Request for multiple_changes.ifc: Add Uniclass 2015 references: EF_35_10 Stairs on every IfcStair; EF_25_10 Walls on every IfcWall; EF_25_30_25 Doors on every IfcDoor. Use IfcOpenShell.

First a look at what the model holds.

```python
import ifcopenshell

model = ifcopenshell.open("multiple_changes.ifc")
print(model.schema)
print("classifications:", [c.Name for c in model.by_type("IfcClassification")])
for ifc_class in ("IfcDoor", "IfcRoof", "IfcStair", "IfcWall", "IfcWindow"):
    print(ifc_class, len(model.by_type(ifc_class)))
```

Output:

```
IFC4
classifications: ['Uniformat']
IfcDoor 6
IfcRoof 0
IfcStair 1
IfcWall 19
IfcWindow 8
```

```python
import ifcopenshell
import ifcopenshell.api.classification

model = ifcopenshell.open("multiple_changes.ifc")

system = ifcopenshell.api.classification.add_classification(model, classification="Uniclass 2015")

codes = {
    "IfcStair": ("EF_35_10", "Stairs"),
    "IfcWall": ("EF_25_10", "Walls"),
    "IfcDoor": ("EF_25_30_25", "Doors"),
}
for ifc_class, (code, name) in codes.items():
    products = model.by_type(ifc_class)
    ifcopenshell.api.classification.add_reference(
        model, products=products, classification=system, identification=code, name=name
    )
    print(code, len(products))

model.write("multiple_changes_updated.ifc")
```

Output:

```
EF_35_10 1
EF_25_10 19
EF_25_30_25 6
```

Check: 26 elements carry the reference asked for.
